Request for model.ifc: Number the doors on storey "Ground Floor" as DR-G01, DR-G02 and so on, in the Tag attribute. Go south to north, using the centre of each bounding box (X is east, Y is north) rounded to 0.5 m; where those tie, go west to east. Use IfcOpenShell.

First a look at what the model holds.

```python
import ifcopenshell
import ifcopenshell.util.element
import ifcopenshell.util.placement

model = ifcopenshell.open("model.ifc")
print(model.schema)
storey = next(s for s in model.by_type("IfcBuildingStorey") if s.Name == "Ground Floor")
doors = [e for e in ifcopenshell.util.element.get_decomposition(storey) if e.is_a("IfcDoor")]
for e in sorted(doors, key=lambda e: e.id()):
    origin = ifcopenshell.util.placement.get_local_placement(e.ObjectPlacement)[:3, 3]
    print(e.id(), e.Tag, e.Name, origin.round(2) + 0.0, sep=" | ")
```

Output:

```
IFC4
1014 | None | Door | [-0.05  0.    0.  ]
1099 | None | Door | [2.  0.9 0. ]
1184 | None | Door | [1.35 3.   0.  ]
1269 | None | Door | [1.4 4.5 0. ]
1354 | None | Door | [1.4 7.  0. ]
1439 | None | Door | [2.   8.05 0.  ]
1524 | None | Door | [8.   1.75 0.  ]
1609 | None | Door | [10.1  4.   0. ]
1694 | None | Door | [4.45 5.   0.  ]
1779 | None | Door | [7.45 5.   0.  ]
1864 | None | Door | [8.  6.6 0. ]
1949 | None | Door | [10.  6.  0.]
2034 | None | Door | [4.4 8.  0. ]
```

```python
import ifcopenshell
import ifcopenshell.geom
import ifcopenshell.util.element
import ifcopenshell.util.shape

model = ifcopenshell.open("model.ifc")
settings = ifcopenshell.geom.settings()
settings.set("use-world-coords", True)


def centre(element):
    shape = ifcopenshell.geom.create_shape(settings, element)
    return ifcopenshell.util.shape.get_bbox_centroid(shape.geometry)


storey = next(s for s in model.by_type("IfcBuildingStorey") if s.Name == "Ground Floor")
doors = [e for e in ifcopenshell.util.element.get_decomposition(storey) if e.is_a("IfcDoor")]

# Insertion points can sit at a corner or the storey origin, so sort by the geometry (in metres).
centres = {e: centre(e) for e in doors}
doors.sort(key=lambda e: (round(centres[e][1] / 0.5), centres[e][0]))

for i, e in enumerate(doors, start=1):
    number = f"DR-G{i:02d}"
    e.Tag = number
    print(e.id(), number)

model.write("model_updated.ifc")
```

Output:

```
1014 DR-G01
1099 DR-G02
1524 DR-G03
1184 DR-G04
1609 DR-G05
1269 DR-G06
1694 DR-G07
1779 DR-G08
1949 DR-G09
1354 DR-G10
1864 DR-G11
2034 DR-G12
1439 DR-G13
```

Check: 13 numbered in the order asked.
